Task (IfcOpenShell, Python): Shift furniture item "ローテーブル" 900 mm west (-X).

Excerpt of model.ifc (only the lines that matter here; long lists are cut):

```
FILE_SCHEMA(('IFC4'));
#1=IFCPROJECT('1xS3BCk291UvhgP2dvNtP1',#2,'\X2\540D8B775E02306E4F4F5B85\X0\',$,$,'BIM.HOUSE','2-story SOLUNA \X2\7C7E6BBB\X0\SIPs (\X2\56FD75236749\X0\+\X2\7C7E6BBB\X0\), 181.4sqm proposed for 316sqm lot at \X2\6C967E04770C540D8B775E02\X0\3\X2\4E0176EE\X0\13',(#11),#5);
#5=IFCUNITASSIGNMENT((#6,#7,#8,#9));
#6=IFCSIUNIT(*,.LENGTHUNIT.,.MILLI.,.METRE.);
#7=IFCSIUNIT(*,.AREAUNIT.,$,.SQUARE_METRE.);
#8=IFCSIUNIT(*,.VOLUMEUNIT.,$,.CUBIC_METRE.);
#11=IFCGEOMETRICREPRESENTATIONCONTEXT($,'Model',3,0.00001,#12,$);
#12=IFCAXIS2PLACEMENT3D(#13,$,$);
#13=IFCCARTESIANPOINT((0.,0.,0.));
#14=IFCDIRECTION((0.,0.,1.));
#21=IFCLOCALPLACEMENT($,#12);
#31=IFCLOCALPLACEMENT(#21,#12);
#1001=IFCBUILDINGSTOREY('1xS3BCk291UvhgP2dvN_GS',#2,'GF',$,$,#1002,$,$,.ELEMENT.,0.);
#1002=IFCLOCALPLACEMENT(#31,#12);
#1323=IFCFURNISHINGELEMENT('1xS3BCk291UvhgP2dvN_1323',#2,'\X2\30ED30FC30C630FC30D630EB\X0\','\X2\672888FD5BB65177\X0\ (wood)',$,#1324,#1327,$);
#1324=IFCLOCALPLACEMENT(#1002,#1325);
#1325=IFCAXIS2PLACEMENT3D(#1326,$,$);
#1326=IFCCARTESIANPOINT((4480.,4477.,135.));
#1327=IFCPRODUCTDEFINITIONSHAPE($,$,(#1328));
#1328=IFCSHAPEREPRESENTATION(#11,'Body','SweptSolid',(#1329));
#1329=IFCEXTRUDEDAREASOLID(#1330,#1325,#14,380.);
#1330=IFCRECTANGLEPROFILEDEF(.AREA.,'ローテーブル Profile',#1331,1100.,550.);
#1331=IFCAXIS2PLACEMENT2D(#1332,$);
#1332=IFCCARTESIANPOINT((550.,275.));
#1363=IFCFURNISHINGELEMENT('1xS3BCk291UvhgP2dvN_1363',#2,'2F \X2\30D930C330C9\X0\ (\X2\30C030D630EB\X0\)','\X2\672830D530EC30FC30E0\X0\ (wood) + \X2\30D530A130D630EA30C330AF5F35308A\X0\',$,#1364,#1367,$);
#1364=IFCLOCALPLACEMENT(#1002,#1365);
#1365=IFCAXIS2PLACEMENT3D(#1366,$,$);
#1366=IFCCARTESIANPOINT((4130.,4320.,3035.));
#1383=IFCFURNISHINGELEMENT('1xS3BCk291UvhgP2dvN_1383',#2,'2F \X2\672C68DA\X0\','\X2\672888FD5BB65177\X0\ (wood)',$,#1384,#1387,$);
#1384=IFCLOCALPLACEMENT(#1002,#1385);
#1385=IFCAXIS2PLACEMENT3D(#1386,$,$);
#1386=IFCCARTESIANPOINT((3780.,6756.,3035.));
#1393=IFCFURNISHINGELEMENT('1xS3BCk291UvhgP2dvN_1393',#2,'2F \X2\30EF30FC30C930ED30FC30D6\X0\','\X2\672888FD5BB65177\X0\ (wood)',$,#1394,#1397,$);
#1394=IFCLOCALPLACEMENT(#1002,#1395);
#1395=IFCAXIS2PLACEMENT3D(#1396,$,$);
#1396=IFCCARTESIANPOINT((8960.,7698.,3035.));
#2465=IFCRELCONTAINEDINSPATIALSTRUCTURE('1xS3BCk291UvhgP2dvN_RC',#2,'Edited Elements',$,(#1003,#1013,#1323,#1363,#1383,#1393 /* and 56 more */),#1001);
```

```python
import ifcopenshell
import ifcopenshell.api.geometry
import ifcopenshell.util.placement

model = ifcopenshell.open("model.ifc")

item = model.by_guid("1xS3BCk291UvhgP2dvN_1323")
matrix = ifcopenshell.util.placement.get_local_placement(item.ObjectPlacement)
matrix[0, 3] -= 900.0
ifcopenshell.api.geometry.edit_object_placement(model, product=item, matrix=matrix, is_si=False)

print(ifcopenshell.util.placement.get_local_placement(item.ObjectPlacement).round(3) + 0.0)

model.write("model_updated.ifc")
```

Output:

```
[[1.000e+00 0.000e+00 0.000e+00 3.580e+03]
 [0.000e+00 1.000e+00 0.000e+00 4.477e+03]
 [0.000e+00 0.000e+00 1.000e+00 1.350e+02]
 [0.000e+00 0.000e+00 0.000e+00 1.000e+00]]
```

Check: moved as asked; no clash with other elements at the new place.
